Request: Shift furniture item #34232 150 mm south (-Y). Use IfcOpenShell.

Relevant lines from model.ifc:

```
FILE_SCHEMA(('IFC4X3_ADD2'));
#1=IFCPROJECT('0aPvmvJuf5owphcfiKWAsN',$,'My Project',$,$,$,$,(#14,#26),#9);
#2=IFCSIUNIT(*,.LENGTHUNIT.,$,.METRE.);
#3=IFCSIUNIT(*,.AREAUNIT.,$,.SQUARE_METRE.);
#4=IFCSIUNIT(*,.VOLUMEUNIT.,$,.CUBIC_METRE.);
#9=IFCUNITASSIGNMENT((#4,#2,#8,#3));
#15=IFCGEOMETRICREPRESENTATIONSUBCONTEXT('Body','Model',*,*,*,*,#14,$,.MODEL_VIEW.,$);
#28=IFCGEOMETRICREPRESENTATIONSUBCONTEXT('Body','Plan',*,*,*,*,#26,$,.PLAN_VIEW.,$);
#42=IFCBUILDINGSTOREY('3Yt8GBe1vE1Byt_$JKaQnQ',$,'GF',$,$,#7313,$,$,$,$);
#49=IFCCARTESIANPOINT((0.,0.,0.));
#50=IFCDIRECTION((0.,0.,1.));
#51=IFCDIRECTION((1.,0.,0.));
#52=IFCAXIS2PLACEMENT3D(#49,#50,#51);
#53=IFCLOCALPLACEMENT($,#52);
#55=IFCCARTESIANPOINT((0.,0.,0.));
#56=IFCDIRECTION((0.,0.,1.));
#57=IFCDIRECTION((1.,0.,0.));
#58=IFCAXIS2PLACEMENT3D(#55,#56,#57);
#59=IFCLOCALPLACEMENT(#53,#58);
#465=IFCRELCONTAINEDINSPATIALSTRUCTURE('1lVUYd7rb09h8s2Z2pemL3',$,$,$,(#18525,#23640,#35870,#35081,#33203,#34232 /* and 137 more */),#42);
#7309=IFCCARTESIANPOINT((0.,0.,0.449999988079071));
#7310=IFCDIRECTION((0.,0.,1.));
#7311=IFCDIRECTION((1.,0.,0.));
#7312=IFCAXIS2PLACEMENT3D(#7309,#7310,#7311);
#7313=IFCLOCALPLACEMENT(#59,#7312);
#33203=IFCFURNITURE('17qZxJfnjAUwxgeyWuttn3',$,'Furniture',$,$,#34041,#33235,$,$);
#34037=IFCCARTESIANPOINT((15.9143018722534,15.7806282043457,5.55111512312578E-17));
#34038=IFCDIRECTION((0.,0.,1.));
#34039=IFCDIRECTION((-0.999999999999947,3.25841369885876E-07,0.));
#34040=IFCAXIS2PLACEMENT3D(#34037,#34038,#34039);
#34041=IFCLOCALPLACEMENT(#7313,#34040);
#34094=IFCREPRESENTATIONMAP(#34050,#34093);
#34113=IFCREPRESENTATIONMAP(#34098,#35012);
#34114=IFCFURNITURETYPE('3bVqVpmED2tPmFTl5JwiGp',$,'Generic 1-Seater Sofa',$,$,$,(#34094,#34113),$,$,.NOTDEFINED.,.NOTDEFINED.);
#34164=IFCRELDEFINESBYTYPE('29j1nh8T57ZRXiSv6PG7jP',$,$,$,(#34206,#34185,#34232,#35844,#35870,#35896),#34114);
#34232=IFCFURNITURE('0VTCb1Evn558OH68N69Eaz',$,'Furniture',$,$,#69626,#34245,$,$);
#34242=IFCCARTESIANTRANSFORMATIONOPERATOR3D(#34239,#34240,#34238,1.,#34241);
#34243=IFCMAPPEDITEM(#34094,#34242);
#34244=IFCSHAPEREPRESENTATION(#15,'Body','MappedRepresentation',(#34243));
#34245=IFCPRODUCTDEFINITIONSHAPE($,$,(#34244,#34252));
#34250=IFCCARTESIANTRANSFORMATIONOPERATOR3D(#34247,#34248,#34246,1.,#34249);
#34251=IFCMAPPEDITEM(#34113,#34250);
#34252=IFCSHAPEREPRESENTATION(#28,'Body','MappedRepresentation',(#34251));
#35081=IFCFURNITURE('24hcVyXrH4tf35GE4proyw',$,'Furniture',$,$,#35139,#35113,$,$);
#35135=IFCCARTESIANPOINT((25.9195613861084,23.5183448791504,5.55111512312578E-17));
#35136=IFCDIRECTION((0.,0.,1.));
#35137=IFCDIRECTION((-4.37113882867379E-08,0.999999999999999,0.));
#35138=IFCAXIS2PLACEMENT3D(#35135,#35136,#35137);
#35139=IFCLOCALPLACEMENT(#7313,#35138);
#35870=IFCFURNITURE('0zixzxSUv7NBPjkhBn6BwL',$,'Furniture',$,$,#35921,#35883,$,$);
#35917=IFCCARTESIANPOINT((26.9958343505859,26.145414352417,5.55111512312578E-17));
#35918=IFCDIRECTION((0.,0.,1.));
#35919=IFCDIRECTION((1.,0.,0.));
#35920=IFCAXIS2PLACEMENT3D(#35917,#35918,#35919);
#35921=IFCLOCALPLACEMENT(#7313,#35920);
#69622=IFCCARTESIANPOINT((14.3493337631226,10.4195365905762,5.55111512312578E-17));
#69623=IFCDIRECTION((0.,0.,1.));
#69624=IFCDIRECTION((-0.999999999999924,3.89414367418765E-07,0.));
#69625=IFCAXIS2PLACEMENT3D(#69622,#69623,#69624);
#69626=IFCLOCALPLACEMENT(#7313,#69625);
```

```python
import ifcopenshell
import ifcopenshell.api.geometry
import ifcopenshell.util.placement
import ifcopenshell.util.unit

model = ifcopenshell.open("model.ifc")
unit_scale = ifcopenshell.util.unit.calculate_unit_scale(model)

item = model.by_guid("0VTCb1Evn558OH68N69Eaz")
matrix = ifcopenshell.util.placement.get_local_placement(item.ObjectPlacement)
matrix[1, 3] -= 0.15 / unit_scale
ifcopenshell.api.geometry.edit_object_placement(model, product=item, matrix=matrix, is_si=False)

print(ifcopenshell.util.placement.get_local_placement(item.ObjectPlacement).round(3) + 0.0)

model.write("model_rev.ifc")
```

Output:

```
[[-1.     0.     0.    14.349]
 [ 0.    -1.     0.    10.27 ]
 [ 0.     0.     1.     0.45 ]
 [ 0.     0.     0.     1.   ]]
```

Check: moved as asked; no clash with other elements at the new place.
